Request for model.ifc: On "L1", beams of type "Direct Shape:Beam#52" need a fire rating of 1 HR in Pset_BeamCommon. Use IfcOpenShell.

First a look at what the model holds.

```python
import ifcopenshell
import ifcopenshell.util.element

model = ifcopenshell.open("model.ifc")
print(model.schema)
storey = next(s for s in model.by_type("IfcBuildingStorey") if s.Name == "L1")
beams = [e for e in ifcopenshell.util.element.get_decomposition(storey) if e.is_a("IfcBeam")]
seen = {}
for e in beams:
    element_type = ifcopenshell.util.element.get_type(e)
    key = (element_type.Name if element_type != e and element_type else None, ifcopenshell.util.element.get_pset(e, "Pset_BeamCommon", "FireRating"))
    seen[key] = seen.get(key, 0) + 1
for (name, value), count in sorted(seen.items(), key=str):
    print(count, "x", name, "|", value)
```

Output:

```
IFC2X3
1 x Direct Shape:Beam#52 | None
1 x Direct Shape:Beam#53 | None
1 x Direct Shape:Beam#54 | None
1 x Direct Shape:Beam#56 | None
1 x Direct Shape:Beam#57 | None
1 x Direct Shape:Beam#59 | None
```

```python
import ifcopenshell
import ifcopenshell.api.pset
import ifcopenshell.util.element

model = ifcopenshell.open("model.ifc")

storey = next(s for s in model.by_type("IfcBuildingStorey") if s.Name == "L1")
beams = [e for e in ifcopenshell.util.element.get_decomposition(storey) if e.is_a("IfcBeam")]

count = 0
for e in beams:
    element_type = ifcopenshell.util.element.get_type(e)
    if element_type in (None, e) or element_type.Name != "Direct Shape:Beam#52":
        continue
    # add_pset returns the element's existing set when there is one.
    pset = ifcopenshell.api.pset.add_pset(model, product=e, name="Pset_BeamCommon")
    ifcopenshell.api.pset.edit_pset(model, pset=pset, properties={"FireRating": "1 HR"})
    count += 1

print(count, "beams updated")

model.write("model_rev.ifc")
```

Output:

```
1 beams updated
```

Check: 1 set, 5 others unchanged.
